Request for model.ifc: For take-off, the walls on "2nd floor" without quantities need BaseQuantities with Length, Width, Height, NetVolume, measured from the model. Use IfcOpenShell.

First a look at what the model holds.

```python
import ifcopenshell
import ifcopenshell.util.element
import ifcopenshell.util.unit

model = ifcopenshell.open("model.ifc")
print(model.schema)
for unit_type in ("LENGTHUNIT", "AREAUNIT", "VOLUMEUNIT"):
    print(unit_type, ifcopenshell.util.unit.calculate_unit_scale(model, unit_type))
storey = next(s for s in model.by_type("IfcBuildingStorey") if s.Name == "2nd floor")
walls = [e for e in ifcopenshell.util.element.get_decomposition(storey) if e.is_a("IfcWall")]
for e in sorted(walls, key=lambda e: e.id()):
    print(e.id(), e.is_a(), e.Name, list(ifcopenshell.util.element.get_psets(e, qtos_only=True)), sep=" | ")
```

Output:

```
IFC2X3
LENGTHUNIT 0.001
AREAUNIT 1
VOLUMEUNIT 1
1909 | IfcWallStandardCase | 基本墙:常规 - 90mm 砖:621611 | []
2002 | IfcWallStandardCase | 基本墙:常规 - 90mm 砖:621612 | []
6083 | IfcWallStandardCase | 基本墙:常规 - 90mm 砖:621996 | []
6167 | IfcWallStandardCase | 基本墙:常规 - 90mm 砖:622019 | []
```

```python
import ifcopenshell
import ifcopenshell.api.pset
import ifcopenshell.geom
import ifcopenshell.util.element
import ifcopenshell.util.shape
import ifcopenshell.util.unit

model = ifcopenshell.open("model.ifc")
unit_scale = ifcopenshell.util.unit.calculate_unit_scale(model)
volume_scale = ifcopenshell.util.unit.calculate_unit_scale(model, "VOLUMEUNIT")
settings = ifcopenshell.geom.settings()

storey = next(s for s in model.by_type("IfcBuildingStorey") if s.Name == "2nd floor")
walls = [e for e in ifcopenshell.util.element.get_decomposition(storey) if e.is_a("IfcWall")]

for e in sorted(walls, key=lambda e: e.id()):
    if ifcopenshell.util.element.get_psets(e, qtos_only=True, should_inherit=False):
        continue
    # Geometry comes back in metres, in the element's own axes.
    shape = ifcopenshell.geom.create_shape(settings, e)
    values = {
        "Length": ifcopenshell.util.shape.get_x(shape.geometry) / unit_scale,
        "Width": ifcopenshell.util.shape.get_y(shape.geometry) / unit_scale,
        "Height": ifcopenshell.util.shape.get_z(shape.geometry) / unit_scale,
        "NetVolume": ifcopenshell.util.shape.get_volume(shape.geometry) / volume_scale,
    }
    qto = ifcopenshell.api.pset.add_qto(model, product=e, name="BaseQuantities")
    ifcopenshell.api.pset.edit_qto(model, qto=qto, properties=values)
    print(e.id(), {k: round(v, 3) for k, v in values.items()})

model.write("model_edited.ifc")
```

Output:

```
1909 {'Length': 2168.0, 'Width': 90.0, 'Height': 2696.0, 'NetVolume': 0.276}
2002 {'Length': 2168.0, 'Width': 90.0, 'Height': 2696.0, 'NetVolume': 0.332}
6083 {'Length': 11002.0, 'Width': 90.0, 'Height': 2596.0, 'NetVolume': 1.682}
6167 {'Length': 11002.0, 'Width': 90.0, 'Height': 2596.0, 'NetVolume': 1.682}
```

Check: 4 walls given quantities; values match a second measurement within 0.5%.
